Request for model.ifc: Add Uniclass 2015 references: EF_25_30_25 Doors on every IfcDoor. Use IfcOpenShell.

First a look at what the model holds.

```python
import ifcopenshell

model = ifcopenshell.open("model.ifc")
print(model.schema)
print("classifications:", [c.Name for c in model.by_type("IfcClassification")])
for ifc_class in ("IfcDoor", "IfcRoof", "IfcStair", "IfcWall", "IfcWindow"):
    print(ifc_class, len(model.by_type(ifc_class)))
```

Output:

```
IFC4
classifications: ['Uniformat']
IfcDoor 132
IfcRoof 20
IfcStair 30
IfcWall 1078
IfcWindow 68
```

```python
import ifcopenshell
import ifcopenshell.api.classification

model = ifcopenshell.open("model.ifc")

system = ifcopenshell.api.classification.add_classification(model, classification="Uniclass 2015")

codes = {
    "IfcDoor": ("EF_25_30_25", "Doors"),
}
for ifc_class, (code, name) in codes.items():
    products = model.by_type(ifc_class)
    ifcopenshell.api.classification.add_reference(
        model, products=products, classification=system, identification=code, name=name
    )
    print(code, len(products))

model.write("model_updated.ifc")
```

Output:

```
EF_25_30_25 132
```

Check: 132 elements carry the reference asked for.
